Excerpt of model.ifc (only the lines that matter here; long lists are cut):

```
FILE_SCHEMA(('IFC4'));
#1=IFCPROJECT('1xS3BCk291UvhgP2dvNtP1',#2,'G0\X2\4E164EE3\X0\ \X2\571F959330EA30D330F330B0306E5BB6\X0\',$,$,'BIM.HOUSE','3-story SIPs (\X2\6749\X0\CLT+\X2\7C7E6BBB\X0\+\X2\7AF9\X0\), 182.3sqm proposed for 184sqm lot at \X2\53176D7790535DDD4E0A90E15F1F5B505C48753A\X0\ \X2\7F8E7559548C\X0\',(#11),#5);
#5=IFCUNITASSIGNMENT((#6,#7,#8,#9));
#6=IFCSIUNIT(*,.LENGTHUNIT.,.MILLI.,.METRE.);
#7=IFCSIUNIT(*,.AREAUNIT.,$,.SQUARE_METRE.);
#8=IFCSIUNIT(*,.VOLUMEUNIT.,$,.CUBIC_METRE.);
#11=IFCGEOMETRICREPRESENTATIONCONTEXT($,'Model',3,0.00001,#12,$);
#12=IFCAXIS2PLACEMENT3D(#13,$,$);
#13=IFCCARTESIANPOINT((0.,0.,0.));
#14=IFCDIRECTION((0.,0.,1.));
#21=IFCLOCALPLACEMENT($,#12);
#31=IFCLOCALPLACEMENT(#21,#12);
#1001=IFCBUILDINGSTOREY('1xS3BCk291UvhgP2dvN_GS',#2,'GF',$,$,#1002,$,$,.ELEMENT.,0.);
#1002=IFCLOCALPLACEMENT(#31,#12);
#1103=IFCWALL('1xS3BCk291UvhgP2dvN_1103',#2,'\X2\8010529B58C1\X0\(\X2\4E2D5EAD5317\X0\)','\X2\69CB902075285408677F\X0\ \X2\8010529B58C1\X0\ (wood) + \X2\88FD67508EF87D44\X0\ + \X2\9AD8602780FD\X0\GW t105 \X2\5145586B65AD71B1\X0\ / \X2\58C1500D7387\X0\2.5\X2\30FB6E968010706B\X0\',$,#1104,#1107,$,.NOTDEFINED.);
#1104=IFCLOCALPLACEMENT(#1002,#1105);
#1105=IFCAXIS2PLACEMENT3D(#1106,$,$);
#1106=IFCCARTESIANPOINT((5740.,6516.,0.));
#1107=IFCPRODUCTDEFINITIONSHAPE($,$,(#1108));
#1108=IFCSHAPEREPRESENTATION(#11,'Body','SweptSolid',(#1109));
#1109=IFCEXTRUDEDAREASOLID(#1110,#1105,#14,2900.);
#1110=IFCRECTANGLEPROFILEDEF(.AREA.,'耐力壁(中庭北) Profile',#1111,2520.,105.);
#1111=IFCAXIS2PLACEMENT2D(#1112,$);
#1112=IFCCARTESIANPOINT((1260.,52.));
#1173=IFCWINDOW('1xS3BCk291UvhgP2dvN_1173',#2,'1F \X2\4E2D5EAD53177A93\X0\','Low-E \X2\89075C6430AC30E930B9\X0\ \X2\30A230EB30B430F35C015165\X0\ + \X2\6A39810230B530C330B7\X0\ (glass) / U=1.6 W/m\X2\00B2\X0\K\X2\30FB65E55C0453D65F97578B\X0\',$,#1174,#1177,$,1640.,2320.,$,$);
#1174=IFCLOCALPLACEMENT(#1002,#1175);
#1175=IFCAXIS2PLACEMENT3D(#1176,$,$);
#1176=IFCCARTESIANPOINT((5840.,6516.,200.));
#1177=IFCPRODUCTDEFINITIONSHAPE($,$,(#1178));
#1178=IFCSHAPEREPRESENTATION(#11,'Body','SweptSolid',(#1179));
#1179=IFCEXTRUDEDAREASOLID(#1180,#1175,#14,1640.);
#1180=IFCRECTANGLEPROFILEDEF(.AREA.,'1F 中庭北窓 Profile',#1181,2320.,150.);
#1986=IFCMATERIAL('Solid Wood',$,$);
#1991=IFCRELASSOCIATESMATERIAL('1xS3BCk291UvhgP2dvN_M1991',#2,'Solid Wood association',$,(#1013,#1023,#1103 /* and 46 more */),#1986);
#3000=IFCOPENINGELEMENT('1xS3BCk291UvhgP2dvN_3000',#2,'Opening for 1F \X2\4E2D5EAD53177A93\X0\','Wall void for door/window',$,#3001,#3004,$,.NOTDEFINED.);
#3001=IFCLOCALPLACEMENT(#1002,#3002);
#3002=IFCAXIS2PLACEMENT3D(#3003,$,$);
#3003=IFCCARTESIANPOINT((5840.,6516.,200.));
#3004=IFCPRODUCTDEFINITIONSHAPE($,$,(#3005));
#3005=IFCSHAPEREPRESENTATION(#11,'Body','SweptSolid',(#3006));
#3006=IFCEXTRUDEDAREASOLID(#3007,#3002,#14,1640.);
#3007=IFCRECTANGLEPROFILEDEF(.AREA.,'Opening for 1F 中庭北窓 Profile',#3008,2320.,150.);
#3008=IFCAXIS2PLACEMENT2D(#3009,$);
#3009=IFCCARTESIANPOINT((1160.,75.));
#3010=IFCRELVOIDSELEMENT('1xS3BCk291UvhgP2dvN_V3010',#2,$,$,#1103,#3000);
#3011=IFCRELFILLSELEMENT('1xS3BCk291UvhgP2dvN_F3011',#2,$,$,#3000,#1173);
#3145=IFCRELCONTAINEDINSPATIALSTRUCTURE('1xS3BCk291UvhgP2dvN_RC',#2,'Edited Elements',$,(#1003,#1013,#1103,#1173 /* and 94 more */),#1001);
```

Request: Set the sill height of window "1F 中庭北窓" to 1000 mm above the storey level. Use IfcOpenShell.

```python
import numpy as np
import ifcopenshell
import ifcopenshell.api.geometry
import ifcopenshell.geom
import ifcopenshell.util.element
import ifcopenshell.util.placement
import ifcopenshell.util.shape
import ifcopenshell.util.unit

model = ifcopenshell.open("model.ifc")
unit_scale = ifcopenshell.util.unit.calculate_unit_scale(model)

window = model.by_id(1173)
opening = window.FillsVoids[0].RelatingOpeningElement
storey = ifcopenshell.util.element.get_container(window, ifc_class="IfcBuildingStorey")
level = ifcopenshell.util.placement.get_local_placement(storey.ObjectPlacement)[2, 3]

# The opening's origin need not be at the sill, so measure its lowest point.
shape = ifcopenshell.geom.create_shape(ifcopenshell.geom.settings(), opening)
bottom = ifcopenshell.util.shape.get_shape_bottom_elevation(shape, shape.geometry) / unit_scale
dz = level + 1000.0 - bottom

shift = np.array([0.0, 0.0, dz])
# The window is not placed relative to its opening, so move both.
for product in (opening, window):
    matrix = ifcopenshell.util.placement.get_local_placement(product.ObjectPlacement)
    matrix[:3, 3] += shift
    ifcopenshell.api.geometry.edit_object_placement(model, product=product, matrix=matrix, is_si=False)

print(f"moved by {dz * unit_scale:+.3f} m")

model.write("model_rev.ifc")
```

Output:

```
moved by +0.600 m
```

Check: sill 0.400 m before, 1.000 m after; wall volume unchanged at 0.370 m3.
